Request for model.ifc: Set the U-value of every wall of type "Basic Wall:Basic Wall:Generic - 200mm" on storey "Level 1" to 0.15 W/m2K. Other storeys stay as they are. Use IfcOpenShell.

First a look at what the model holds.

```python
import ifcopenshell
import ifcopenshell.util.element

model = ifcopenshell.open("model.ifc")
print(model.schema)
storey = next(s for s in model.by_type("IfcBuildingStorey") if s.Name == "Level 1")
walls = [e for e in ifcopenshell.util.element.get_decomposition(storey) if e.is_a("IfcWall")]
seen = {}
for e in walls:
    element_type = ifcopenshell.util.element.get_type(e)
    key = (element_type.Name if element_type != e and element_type else None, ifcopenshell.util.element.get_pset(e, "Pset_WallCommon", "ThermalTransmittance"))
    seen[key] = seen.get(key, 0) + 1
for (name, value), count in sorted(seen.items(), key=str):
    print(count, "x", name, "|", value)
```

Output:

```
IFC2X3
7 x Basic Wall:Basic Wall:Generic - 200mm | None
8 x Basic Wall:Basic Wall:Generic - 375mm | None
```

```python
import ifcopenshell
import ifcopenshell.api.pset
import ifcopenshell.util.element

model = ifcopenshell.open("model.ifc")

storey = next(s for s in model.by_type("IfcBuildingStorey") if s.Name == "Level 1")
walls = [e for e in ifcopenshell.util.element.get_decomposition(storey) if e.is_a("IfcWall")]

count = 0
for e in walls:
    element_type = ifcopenshell.util.element.get_type(e)
    if element_type in (None, e) or element_type.Name != "Basic Wall:Basic Wall:Generic - 200mm":
        continue
    # add_pset returns the element's existing set when there is one.
    pset = ifcopenshell.api.pset.add_pset(model, product=e, name="Pset_WallCommon")
    ifcopenshell.api.pset.edit_pset(model, pset=pset, properties={"ThermalTransmittance": 0.15})
    count += 1

print(count, "walls updated")

model.write("model_updated.ifc")
```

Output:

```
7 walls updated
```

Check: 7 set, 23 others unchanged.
